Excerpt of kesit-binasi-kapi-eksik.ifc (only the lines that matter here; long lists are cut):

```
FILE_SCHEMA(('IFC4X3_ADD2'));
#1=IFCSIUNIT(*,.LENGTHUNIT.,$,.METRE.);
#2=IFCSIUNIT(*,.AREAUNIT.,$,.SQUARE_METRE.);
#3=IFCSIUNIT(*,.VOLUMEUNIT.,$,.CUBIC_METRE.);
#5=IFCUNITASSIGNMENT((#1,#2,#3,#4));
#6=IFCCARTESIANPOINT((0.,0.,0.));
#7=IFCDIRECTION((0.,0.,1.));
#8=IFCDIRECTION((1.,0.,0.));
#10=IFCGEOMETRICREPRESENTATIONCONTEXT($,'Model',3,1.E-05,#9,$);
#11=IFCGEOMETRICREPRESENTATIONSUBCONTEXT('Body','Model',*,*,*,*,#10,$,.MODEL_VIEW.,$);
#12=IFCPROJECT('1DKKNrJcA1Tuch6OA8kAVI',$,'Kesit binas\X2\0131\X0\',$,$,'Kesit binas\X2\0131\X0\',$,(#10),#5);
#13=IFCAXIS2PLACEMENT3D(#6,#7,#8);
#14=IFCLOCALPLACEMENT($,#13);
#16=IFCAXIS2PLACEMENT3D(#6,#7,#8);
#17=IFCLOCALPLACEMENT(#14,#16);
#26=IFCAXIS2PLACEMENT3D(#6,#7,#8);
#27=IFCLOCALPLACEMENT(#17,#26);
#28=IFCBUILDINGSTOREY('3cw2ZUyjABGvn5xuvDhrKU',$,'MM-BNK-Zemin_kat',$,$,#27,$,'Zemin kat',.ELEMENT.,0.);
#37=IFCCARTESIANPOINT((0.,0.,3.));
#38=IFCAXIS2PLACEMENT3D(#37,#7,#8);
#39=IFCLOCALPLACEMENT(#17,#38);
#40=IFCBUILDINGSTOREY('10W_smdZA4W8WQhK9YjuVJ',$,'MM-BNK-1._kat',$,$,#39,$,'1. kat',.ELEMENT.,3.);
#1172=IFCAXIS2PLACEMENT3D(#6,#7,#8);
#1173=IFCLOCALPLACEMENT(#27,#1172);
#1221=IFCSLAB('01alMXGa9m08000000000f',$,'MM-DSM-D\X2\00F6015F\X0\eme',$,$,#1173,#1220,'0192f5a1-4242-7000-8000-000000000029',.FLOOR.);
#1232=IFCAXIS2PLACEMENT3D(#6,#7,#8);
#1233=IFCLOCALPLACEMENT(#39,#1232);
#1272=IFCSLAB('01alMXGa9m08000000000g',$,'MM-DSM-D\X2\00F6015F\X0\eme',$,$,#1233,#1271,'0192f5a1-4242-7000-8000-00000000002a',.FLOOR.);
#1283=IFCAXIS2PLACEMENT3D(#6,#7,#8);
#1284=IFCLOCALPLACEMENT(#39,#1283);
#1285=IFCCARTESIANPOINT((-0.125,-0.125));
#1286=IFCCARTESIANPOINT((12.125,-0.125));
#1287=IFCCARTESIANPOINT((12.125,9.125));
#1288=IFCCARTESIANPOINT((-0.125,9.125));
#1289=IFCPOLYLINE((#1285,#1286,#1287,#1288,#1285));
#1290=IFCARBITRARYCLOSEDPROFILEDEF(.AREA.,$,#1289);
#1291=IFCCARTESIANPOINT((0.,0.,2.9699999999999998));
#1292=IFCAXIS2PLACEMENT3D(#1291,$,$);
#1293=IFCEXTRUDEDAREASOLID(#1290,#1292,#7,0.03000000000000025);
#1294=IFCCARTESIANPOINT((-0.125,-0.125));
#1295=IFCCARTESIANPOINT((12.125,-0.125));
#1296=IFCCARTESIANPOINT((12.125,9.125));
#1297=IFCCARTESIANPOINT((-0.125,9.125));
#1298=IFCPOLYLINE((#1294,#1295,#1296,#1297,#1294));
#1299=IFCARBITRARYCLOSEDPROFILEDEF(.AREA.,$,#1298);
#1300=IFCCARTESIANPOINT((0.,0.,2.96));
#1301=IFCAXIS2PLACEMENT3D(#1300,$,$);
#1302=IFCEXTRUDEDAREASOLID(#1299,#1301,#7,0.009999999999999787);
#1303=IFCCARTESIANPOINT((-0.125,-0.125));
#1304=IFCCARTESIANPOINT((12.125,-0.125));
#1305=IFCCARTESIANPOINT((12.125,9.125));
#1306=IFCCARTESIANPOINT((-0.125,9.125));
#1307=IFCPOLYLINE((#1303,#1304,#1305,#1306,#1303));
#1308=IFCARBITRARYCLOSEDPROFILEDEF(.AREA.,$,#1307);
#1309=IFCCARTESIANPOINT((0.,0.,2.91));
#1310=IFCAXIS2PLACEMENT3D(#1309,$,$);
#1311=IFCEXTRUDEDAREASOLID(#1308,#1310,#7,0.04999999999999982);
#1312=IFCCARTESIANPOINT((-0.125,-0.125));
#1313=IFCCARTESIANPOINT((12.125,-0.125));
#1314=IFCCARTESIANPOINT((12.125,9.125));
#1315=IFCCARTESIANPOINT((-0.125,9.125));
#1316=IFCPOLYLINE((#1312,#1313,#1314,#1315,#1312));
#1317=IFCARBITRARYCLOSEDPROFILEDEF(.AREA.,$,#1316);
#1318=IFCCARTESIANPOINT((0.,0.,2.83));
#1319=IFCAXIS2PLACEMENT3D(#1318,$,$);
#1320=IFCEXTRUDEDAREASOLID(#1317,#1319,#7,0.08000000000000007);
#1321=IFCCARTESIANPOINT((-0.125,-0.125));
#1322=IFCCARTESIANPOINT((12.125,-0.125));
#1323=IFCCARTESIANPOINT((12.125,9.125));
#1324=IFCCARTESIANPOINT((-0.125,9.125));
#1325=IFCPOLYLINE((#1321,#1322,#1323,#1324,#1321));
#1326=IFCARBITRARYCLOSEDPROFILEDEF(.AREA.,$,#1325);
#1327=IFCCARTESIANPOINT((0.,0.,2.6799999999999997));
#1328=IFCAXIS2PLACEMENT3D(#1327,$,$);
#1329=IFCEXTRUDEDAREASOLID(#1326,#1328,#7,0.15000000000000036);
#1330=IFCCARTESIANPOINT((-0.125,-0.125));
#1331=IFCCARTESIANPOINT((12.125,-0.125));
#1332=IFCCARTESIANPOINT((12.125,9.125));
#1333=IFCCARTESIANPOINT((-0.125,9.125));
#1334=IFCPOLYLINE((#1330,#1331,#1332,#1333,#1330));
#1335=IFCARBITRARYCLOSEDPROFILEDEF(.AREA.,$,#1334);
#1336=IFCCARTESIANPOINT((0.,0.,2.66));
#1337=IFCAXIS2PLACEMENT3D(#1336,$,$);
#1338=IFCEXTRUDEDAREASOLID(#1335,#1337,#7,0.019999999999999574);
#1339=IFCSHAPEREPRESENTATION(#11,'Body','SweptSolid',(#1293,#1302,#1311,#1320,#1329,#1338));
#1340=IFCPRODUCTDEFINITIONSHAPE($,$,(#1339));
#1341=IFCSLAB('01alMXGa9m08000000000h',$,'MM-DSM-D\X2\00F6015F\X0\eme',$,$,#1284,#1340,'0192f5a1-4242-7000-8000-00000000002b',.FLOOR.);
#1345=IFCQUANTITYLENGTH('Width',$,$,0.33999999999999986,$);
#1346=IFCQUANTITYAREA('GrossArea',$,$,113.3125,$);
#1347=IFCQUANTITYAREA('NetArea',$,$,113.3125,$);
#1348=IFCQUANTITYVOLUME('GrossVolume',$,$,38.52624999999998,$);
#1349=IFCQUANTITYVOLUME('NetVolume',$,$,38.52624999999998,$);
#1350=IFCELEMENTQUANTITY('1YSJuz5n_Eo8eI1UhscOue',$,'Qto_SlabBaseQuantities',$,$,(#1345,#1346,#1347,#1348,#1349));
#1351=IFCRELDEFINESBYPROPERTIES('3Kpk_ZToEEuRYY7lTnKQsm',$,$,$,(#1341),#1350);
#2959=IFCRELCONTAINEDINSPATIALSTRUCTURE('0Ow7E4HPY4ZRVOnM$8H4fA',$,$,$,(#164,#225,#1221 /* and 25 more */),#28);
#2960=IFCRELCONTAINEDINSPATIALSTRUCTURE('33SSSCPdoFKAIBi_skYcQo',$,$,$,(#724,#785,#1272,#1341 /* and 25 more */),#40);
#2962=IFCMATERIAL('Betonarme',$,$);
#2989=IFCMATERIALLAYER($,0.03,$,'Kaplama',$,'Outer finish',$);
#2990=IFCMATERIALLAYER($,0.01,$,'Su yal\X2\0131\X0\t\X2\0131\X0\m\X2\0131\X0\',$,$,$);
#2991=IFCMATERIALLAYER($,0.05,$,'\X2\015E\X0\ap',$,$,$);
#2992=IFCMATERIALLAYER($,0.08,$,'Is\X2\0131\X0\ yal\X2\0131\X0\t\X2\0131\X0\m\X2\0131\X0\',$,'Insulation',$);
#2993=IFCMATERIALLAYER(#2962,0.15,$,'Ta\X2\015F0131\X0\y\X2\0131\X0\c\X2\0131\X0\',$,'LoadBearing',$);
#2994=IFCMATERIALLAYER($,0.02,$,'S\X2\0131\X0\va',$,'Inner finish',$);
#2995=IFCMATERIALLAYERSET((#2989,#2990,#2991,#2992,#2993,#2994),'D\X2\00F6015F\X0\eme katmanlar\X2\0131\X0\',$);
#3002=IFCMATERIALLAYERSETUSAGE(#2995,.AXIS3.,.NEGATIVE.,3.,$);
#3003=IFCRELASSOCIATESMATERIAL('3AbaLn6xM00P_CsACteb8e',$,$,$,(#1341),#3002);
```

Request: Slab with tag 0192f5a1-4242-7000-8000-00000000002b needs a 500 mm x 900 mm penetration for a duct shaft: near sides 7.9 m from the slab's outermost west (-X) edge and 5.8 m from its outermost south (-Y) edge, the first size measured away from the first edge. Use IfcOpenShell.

```python
import numpy as np
import ifcopenshell
import ifcopenshell.api.feature
import ifcopenshell.api.geometry
import ifcopenshell.api.pset
import ifcopenshell.api.root
import ifcopenshell.geom
import ifcopenshell.util.element
import ifcopenshell.util.placement
import ifcopenshell.util.representation
import ifcopenshell.util.shape
import ifcopenshell.util.unit

model = ifcopenshell.open("kesit-binasi-kapi-eksik.ifc")
unit_scale = ifcopenshell.util.unit.calculate_unit_scale(model)
area_scale = ifcopenshell.util.unit.calculate_unit_scale(model, "AREAUNIT")
volume_scale = ifcopenshell.util.unit.calculate_unit_scale(model, "VOLUMEUNIT")
settings = ifcopenshell.geom.settings()


def volume(element):
    """Net volume in cubic metres, openings subtracted."""
    shape = ifcopenshell.geom.create_shape(settings, element)
    return ifcopenshell.util.shape.get_volume(shape.geometry)


slab = model.by_guid("01alMXGa9m08000000000h")
before = volume(slab)

# Extent in the slab's own axes, in metres. The edges named are its -X and -Y sides.
slab_shape = ifcopenshell.geom.create_shape(settings, slab)
vertices = ifcopenshell.util.shape.get_vertices(slab_shape.geometry)
x_min, y_min, bottom = vertices.min(axis=0)
top = vertices[:, 2].max()

opening = ifcopenshell.api.root.create_entity(model, ifc_class="IfcOpeningElement", name="Duct shaft opening", predefined_type="OPENING")
context = ifcopenshell.util.representation.get_context(model, "Model", "Body", "MODEL_VIEW")
width, depth = 0.5, 0.9
outline = [(0.0, 0.0), (width, 0.0), (width, depth), (0.0, depth), (0.0, 0.0)]
# Overshoot both faces by 50 mm so the cut is clean.
shape = ifcopenshell.api.geometry.add_slab_representation(
    model, context=context, depth=top - bottom + 0.1, polyline=outline
)
ifcopenshell.api.geometry.assign_representation(model, product=opening, representation=shape)

matrix = ifcopenshell.util.placement.get_local_placement(slab.ObjectPlacement)
matrix[:, 3] = matrix @ np.append(np.array([x_min + 7.9, y_min + 5.8, bottom - 0.05]) / unit_scale, 1.0)
ifcopenshell.api.geometry.edit_object_placement(model, product=opening, matrix=matrix, is_si=False)
ifcopenshell.api.feature.add_feature(model, feature=opening, element=slab)

after = volume(slab)

# Update the slab's stored quantities.
qto = model.by_id(ifcopenshell.util.element.get_pset(slab, "Qto_SlabBaseQuantities", should_inherit=False)["id"])
ifcopenshell.api.pset.edit_qto(model, qto=qto, properties={
    "NetArea": after / (top - bottom) / area_scale,
    "NetVolume": after / volume_scale,
})

print(f"slab volume {before:.3f} -> {after:.3f} m3")

model.write("kesit-binasi-kapi-eksik_rev.ifc")
```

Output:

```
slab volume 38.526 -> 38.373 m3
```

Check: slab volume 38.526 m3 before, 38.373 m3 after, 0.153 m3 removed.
